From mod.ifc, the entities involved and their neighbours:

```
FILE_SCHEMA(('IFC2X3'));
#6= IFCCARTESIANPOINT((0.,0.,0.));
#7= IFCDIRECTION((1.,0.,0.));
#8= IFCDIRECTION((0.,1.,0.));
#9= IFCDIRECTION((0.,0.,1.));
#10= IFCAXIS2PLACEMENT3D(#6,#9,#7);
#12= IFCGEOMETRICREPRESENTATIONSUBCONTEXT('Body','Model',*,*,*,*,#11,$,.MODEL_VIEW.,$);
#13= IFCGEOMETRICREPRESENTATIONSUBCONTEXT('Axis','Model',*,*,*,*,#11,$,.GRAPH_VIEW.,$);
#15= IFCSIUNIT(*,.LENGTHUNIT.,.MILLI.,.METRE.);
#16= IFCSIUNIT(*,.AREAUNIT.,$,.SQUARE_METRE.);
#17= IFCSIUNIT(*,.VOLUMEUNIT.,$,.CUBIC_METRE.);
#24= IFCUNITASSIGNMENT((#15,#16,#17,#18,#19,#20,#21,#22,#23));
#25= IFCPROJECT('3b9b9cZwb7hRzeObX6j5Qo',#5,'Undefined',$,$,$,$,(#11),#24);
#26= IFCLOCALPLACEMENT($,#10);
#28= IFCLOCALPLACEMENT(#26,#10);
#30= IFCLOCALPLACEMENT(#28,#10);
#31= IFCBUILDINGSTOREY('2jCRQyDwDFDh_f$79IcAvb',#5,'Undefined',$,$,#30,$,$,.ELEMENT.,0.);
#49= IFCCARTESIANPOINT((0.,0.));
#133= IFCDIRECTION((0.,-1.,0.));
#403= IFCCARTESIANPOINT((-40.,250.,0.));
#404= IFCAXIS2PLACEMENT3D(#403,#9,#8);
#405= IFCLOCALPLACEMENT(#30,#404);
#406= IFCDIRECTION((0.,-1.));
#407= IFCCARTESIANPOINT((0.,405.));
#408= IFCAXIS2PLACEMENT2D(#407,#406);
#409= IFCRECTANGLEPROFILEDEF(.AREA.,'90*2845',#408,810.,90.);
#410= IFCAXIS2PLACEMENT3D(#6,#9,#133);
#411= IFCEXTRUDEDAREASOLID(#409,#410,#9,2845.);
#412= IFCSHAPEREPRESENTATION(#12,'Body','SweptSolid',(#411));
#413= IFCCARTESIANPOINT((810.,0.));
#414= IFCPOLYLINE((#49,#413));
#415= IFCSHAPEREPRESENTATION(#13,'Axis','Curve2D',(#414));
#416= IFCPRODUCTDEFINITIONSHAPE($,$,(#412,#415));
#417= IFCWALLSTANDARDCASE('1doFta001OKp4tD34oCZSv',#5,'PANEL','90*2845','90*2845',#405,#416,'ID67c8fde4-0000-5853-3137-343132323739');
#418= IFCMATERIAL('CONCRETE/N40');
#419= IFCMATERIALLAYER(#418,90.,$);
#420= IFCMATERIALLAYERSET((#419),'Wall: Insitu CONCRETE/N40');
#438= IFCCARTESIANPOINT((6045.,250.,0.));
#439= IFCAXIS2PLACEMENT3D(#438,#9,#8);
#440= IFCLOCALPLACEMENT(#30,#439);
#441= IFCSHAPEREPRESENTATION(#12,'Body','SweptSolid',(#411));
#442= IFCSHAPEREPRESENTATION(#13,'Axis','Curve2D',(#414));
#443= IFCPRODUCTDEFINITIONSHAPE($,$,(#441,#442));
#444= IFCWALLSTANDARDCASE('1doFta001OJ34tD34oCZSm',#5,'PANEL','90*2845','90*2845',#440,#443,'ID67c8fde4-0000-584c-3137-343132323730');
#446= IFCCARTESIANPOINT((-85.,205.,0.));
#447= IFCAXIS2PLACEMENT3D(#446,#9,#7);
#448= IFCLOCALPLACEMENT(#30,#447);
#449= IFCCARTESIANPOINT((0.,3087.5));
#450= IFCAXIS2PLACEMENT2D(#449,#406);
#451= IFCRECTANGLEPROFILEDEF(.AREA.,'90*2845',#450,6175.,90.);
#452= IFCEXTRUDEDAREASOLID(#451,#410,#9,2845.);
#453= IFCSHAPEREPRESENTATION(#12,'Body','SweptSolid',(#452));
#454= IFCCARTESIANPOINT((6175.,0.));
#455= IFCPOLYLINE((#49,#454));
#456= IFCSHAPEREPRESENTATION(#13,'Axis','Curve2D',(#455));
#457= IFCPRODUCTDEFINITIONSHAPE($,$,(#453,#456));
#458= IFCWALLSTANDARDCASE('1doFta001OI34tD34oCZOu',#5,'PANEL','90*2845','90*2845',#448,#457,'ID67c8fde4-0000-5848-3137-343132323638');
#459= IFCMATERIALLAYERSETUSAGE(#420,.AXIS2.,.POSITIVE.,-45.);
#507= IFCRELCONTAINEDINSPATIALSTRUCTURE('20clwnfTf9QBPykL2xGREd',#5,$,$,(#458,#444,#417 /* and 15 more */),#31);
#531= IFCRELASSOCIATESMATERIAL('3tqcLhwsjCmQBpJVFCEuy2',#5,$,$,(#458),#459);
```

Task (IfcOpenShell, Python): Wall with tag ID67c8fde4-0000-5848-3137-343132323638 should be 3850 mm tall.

```python
import ifcopenshell
import ifcopenshell.geom
import ifcopenshell.util.representation
import ifcopenshell.util.shape
import ifcopenshell.util.unit

model = ifcopenshell.open("mod.ifc")
unit_scale = ifcopenshell.util.unit.calculate_unit_scale(model)
settings = ifcopenshell.geom.settings()


def volume(element):
    """Net volume in cubic metres, openings subtracted."""
    shape = ifcopenshell.geom.create_shape(settings, element)
    return ifcopenshell.util.shape.get_volume(shape.geometry)


wall = model.by_guid("1doFta001OI34tD34oCZOu")
before = volume(wall)

body = ifcopenshell.util.representation.get_representation(wall, "Model", "Body")
solid = body.Items[0]
old_height = solid.Depth
solid.Depth = 3.85 / unit_scale
after = volume(wall)

print(f"height {old_height:g} -> {solid.Depth:g}, volume {before:.3f} -> {after:.3f} m3")

model.write("mod_updated.ifc")
```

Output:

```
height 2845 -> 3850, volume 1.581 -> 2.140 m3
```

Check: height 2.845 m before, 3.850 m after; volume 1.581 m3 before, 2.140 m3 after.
